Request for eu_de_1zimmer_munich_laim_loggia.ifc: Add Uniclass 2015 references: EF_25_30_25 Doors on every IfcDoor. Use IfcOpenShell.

First a look at what the model holds.

```python
import ifcopenshell

model = ifcopenshell.open("eu_de_1zimmer_munich_laim_loggia.ifc")
print(model.schema)
print("classifications:", [c.Name for c in model.by_type("IfcClassification")])
for ifc_class in ("IfcDoor", "IfcRoof", "IfcStair", "IfcWall", "IfcWindow"):
    print(ifc_class, len(model.by_type(ifc_class)))
```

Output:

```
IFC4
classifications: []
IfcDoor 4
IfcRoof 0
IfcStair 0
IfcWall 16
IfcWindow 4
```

```python
import ifcopenshell
import ifcopenshell.api.classification

model = ifcopenshell.open("eu_de_1zimmer_munich_laim_loggia.ifc")

system = ifcopenshell.api.classification.add_classification(model, classification="Uniclass 2015")

codes = {
    "IfcDoor": ("EF_25_30_25", "Doors"),
}
for ifc_class, (code, name) in codes.items():
    products = model.by_type(ifc_class)
    ifcopenshell.api.classification.add_reference(
        model, products=products, classification=system, identification=code, name=name
    )
    print(code, len(products))

model.write("eu_de_1zimmer_munich_laim_loggia_updated.ifc")
```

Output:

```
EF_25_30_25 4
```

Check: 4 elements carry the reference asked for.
